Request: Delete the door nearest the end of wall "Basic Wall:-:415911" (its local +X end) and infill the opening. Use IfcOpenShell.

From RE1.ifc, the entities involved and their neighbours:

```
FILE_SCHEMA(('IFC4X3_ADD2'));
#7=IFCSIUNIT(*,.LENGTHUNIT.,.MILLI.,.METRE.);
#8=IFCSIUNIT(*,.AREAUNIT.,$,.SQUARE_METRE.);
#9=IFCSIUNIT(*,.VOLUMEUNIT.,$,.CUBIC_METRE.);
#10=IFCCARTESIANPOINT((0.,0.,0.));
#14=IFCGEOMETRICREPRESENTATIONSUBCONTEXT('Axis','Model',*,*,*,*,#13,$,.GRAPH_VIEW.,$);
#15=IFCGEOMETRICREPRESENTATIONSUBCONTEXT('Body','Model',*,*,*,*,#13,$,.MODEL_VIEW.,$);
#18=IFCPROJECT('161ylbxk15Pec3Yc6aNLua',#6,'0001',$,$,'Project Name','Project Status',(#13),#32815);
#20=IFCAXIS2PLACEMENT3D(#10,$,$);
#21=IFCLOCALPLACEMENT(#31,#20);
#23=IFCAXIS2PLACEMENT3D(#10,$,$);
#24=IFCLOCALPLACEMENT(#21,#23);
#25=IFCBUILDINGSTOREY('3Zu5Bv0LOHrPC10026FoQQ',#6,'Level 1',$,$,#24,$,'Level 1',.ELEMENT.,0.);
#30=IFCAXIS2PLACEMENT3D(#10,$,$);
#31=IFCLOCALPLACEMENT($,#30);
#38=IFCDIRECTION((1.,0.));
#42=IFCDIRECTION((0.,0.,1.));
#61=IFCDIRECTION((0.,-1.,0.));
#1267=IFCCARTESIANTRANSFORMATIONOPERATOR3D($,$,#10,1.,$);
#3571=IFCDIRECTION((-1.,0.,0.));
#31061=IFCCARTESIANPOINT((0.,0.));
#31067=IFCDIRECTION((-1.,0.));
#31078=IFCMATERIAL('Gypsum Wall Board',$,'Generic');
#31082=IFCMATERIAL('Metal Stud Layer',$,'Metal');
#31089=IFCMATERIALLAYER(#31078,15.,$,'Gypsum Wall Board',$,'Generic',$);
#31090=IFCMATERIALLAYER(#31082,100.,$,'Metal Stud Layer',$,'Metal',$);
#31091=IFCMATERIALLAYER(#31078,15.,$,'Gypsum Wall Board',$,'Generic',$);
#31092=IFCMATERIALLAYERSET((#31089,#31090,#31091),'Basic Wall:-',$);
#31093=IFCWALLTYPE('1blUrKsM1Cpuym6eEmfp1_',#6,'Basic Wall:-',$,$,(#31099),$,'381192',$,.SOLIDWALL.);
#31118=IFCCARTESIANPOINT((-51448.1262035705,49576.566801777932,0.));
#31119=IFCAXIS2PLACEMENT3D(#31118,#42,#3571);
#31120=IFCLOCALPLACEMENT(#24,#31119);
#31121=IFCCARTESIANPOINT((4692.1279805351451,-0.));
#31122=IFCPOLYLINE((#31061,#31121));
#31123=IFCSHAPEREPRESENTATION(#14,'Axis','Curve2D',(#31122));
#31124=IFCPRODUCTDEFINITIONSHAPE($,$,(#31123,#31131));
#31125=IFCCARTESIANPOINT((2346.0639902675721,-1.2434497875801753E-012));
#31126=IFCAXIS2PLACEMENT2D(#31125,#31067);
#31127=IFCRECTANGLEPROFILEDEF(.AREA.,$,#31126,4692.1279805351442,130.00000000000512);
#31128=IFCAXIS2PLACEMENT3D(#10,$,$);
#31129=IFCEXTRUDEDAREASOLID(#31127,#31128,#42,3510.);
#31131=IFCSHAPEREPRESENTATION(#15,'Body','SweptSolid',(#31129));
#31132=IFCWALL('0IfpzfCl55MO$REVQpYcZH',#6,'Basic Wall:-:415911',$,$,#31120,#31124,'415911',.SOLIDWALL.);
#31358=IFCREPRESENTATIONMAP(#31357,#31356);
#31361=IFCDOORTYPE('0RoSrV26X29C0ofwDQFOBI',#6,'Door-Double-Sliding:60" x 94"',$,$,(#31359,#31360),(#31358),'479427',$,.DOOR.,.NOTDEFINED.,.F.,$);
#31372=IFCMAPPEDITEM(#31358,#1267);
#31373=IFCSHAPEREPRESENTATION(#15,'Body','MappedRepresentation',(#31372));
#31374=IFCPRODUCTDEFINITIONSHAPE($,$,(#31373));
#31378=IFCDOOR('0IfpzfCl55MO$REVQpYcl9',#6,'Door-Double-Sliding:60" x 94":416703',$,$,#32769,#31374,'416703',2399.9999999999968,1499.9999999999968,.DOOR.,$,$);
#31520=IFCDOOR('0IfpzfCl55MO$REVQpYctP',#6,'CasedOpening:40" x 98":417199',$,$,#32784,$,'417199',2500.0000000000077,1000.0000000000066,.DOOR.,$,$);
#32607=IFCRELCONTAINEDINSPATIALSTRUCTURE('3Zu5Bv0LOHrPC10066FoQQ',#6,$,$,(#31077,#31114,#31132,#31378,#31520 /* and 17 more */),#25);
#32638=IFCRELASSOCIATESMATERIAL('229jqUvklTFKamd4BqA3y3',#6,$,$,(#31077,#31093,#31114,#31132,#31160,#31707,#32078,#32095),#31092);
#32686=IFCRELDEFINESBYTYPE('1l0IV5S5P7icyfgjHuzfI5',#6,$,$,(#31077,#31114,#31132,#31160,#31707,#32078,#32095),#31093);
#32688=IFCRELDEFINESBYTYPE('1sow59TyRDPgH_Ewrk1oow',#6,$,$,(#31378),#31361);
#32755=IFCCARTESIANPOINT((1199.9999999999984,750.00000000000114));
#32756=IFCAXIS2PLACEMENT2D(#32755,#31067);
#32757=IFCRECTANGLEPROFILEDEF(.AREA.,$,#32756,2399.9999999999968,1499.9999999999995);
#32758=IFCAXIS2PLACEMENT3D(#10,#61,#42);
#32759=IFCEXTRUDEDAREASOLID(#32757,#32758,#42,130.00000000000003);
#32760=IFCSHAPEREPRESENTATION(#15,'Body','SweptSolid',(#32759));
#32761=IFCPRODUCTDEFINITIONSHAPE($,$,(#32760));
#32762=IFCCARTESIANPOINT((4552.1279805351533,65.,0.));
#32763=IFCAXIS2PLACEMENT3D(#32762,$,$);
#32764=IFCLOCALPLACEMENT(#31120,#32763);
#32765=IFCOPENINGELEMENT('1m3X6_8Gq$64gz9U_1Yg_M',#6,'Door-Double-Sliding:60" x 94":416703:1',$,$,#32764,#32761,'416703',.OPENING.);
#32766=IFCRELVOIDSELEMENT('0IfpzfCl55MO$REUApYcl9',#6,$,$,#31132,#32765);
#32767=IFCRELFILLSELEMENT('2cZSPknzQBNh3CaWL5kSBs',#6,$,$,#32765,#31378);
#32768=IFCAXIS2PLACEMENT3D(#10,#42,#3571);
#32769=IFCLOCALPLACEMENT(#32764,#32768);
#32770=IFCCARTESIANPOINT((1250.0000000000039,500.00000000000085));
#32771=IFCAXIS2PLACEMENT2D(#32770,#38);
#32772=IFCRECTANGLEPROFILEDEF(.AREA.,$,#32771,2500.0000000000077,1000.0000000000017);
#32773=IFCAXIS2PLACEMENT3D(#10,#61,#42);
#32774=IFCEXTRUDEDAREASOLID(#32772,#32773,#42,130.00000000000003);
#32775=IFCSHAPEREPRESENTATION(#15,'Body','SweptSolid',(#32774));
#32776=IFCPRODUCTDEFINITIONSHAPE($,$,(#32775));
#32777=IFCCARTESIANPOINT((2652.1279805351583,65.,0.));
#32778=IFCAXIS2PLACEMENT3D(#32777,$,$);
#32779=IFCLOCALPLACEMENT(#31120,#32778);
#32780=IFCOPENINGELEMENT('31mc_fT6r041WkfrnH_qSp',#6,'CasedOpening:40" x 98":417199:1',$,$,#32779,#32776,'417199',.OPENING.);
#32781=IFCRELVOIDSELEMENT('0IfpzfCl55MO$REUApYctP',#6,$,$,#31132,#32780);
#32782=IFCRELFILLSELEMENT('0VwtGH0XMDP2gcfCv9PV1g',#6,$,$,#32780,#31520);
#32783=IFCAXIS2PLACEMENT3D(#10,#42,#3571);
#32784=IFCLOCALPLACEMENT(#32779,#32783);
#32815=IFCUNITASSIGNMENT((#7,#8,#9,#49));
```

```python
import ifcopenshell
import ifcopenshell.api.feature
import ifcopenshell.api.root
import ifcopenshell.geom
import ifcopenshell.util.shape

model = ifcopenshell.open("RE1.ifc")
settings = ifcopenshell.geom.settings()


def volume(element):
    """Net volume in cubic metres, openings subtracted."""
    shape = ifcopenshell.geom.create_shape(settings, element)
    return ifcopenshell.util.shape.get_volume(shape.geometry)


door = model.by_id(31378)
opening = door.FillsVoids[0].RelatingOpeningElement
wall = opening.VoidsElements[0].RelatingBuildingElement
before = volume(wall)

ifcopenshell.api.root.remove_product(model, product=door)
ifcopenshell.api.feature.remove_feature(model, feature=opening)

after = volume(wall)

print(f"wall volume {before:.3f} -> {after:.3f} m3")

model.write("RE1_rev.ifc")
```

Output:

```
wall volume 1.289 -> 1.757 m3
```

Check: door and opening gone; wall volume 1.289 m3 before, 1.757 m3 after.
